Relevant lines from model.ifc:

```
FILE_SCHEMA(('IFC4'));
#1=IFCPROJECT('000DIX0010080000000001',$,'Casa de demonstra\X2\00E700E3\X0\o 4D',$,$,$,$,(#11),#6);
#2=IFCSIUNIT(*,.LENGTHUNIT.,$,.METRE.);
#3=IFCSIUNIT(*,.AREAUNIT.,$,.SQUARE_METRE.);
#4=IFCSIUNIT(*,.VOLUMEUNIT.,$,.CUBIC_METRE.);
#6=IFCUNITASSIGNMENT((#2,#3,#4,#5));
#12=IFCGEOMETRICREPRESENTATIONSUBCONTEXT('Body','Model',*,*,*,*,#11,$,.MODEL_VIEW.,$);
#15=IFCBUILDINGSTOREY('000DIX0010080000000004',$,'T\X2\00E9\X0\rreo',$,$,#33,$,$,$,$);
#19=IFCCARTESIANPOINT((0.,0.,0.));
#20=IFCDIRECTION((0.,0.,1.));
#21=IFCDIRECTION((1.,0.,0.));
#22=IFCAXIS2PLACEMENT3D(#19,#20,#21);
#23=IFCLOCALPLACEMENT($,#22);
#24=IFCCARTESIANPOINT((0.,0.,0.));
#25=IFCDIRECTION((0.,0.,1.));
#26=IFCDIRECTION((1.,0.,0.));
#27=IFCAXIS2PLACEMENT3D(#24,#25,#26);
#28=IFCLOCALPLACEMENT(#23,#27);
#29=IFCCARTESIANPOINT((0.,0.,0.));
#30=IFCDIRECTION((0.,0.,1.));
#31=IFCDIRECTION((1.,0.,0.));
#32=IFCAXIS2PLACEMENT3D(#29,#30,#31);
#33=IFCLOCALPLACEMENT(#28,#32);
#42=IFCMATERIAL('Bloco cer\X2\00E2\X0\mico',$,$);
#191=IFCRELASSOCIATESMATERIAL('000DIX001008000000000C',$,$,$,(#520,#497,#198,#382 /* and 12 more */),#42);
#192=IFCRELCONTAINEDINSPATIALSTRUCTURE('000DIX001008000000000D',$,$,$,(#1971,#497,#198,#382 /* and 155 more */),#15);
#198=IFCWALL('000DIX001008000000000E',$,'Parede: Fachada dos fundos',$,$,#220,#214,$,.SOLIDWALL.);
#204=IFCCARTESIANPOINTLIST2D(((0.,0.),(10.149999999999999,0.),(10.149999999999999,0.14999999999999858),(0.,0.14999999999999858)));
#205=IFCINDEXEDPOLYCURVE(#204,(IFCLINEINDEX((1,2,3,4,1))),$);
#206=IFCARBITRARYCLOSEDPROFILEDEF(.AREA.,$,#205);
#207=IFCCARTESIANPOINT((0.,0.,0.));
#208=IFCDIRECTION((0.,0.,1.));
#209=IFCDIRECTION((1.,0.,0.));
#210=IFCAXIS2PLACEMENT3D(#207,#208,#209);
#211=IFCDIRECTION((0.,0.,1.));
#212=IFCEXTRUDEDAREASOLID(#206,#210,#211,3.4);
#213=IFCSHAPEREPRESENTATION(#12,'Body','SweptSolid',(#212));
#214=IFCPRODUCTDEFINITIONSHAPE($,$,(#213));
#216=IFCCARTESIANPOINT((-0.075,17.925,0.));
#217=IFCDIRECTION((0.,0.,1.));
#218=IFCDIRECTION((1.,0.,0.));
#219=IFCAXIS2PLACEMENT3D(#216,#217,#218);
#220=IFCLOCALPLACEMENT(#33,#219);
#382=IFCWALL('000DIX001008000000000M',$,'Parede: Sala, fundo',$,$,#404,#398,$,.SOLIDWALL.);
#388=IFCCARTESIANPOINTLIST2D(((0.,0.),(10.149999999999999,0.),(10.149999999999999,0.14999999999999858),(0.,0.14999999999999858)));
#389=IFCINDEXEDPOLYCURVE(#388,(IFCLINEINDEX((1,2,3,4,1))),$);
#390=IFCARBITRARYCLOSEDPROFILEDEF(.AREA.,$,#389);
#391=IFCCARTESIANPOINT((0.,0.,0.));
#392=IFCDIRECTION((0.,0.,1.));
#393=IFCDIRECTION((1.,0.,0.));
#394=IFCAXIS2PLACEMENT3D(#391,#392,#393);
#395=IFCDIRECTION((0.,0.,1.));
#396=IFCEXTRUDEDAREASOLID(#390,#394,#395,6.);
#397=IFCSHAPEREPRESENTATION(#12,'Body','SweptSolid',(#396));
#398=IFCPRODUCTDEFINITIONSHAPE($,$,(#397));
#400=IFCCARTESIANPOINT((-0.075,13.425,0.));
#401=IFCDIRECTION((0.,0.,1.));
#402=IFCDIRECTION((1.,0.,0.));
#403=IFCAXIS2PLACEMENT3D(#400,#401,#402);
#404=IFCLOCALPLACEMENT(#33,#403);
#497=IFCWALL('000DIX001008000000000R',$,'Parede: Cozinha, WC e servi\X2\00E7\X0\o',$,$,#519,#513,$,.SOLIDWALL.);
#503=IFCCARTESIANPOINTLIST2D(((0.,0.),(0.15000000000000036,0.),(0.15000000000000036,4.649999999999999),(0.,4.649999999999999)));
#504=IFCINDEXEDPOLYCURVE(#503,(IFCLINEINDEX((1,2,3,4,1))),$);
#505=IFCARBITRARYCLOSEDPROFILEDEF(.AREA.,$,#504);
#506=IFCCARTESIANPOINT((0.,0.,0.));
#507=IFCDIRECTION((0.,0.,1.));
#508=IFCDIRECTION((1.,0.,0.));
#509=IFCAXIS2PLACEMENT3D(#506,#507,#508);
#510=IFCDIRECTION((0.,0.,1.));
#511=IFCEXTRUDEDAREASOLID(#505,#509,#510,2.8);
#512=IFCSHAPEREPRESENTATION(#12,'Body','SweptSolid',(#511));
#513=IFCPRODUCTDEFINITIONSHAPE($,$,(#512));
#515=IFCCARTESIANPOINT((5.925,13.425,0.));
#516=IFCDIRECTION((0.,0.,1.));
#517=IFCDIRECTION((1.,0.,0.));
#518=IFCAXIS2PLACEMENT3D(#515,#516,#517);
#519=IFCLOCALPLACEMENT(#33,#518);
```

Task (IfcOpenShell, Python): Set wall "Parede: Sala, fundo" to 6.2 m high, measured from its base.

```python
import ifcopenshell
import ifcopenshell.geom
import ifcopenshell.util.representation
import ifcopenshell.util.shape

model = ifcopenshell.open("model.ifc")
settings = ifcopenshell.geom.settings()


def volume(element):
    """Net volume in cubic metres, openings subtracted."""
    shape = ifcopenshell.geom.create_shape(settings, element)
    return ifcopenshell.util.shape.get_volume(shape.geometry)


wall = model.by_id(382)
before = volume(wall)

body = ifcopenshell.util.representation.get_representation(wall, "Model", "Body")
solid = body.Items[0]
old_height = solid.Depth
solid.Depth = 6.2
after = volume(wall)

print(f"height {old_height:g} -> {solid.Depth:g}, volume {before:.3f} -> {after:.3f} m3")

model.write("model_v2.ifc")
```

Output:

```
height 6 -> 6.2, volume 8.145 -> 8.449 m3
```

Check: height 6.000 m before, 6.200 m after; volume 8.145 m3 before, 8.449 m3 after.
